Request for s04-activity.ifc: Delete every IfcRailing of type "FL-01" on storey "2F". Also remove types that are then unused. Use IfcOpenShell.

First a look at what the model holds.

```python
import ifcopenshell
import ifcopenshell.util.element

model = ifcopenshell.open("s04-activity.ifc")
print(model.schema)
storey = next(s for s in model.by_type("IfcBuildingStorey") if s.Name == "2F")
railings = [e for e in ifcopenshell.util.element.get_decomposition(storey) if e.is_a("IfcRailing")]
seen = {}
for e in railings:
    element_type = ifcopenshell.util.element.get_type(e)
    name = element_type.Name if element_type not in (None, e) else None
    seen[name] = seen.get(name, 0) + 1
for name, count in sorted(seen.items(), key=str):
    print(count, "x", name)
```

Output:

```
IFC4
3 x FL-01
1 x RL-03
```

```python
import ifcopenshell
import ifcopenshell.api.root
import ifcopenshell.util.element

model = ifcopenshell.open("s04-activity.ifc")

storey = next(s for s in model.by_type("IfcBuildingStorey") if s.Name == "2F")
railings = [e for e in ifcopenshell.util.element.get_decomposition(storey) if e.is_a("IfcRailing")]
targets = [e for e in railings if (t := ifcopenshell.util.element.get_type(e)) not in (None, e) and t.Name == "FL-01"]
types = {ifcopenshell.util.element.get_type(e) for e in targets} - {None, *targets}

for e in targets:
    ifcopenshell.api.root.remove_product(model, product=e)
print(len(targets), "removed")

unused = [t for t in types if not ifcopenshell.util.element.get_types(t)]
for t in unused:
    ifcopenshell.api.root.remove_product(model, product=t)
print(len(unused), "unused types removed")

model.write("s04-activity_updated.ifc")
```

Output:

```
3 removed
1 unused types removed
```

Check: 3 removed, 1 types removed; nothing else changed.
